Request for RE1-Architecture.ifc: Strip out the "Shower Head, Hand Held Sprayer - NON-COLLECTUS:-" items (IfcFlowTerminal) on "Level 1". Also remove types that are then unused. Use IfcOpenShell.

First a look at what the model holds.

```python
import ifcopenshell
import ifcopenshell.util.element

model = ifcopenshell.open("RE1-Architecture.ifc")
print(model.schema)
storey = next(s for s in model.by_type("IfcBuildingStorey") if s.Name == "Level 1")
terminals = [e for e in ifcopenshell.util.element.get_decomposition(storey) if e.is_a("IfcFlowTerminal")]
seen = {}
for e in terminals:
    element_type = ifcopenshell.util.element.get_type(e)
    name = element_type.Name if element_type not in (None, e) else None
    seen[name] = seen.get(name, 0) + 1
for name, count in sorted(seen.items(), key=str):
    print(count, "x", name)
```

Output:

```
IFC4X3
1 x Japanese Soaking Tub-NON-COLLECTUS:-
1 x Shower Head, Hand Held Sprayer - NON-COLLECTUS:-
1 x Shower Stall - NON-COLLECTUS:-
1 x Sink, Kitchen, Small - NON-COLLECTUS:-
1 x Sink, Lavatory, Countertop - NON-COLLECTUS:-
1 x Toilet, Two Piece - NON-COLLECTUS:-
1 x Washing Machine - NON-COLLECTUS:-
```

```python
import ifcopenshell
import ifcopenshell.api.root
import ifcopenshell.util.element

model = ifcopenshell.open("RE1-Architecture.ifc")

storey = next(s for s in model.by_type("IfcBuildingStorey") if s.Name == "Level 1")
terminals = [e for e in ifcopenshell.util.element.get_decomposition(storey) if e.is_a("IfcFlowTerminal")]
targets = [e for e in terminals if (t := ifcopenshell.util.element.get_type(e)) not in (None, e) and t.Name == "Shower Head, Hand Held Sprayer - NON-COLLECTUS:-"]
types = {ifcopenshell.util.element.get_type(e) for e in targets} - {None, *targets}

for e in targets:
    ifcopenshell.api.root.remove_product(model, product=e)
print(len(targets), "removed")

unused = [t for t in types if not ifcopenshell.util.element.get_types(t)]
for t in unused:
    ifcopenshell.api.root.remove_product(model, product=t)
print(len(unused), "unused types removed")

model.write("RE1-Architecture_v2.ifc")
```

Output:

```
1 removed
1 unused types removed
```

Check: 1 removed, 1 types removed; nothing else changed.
